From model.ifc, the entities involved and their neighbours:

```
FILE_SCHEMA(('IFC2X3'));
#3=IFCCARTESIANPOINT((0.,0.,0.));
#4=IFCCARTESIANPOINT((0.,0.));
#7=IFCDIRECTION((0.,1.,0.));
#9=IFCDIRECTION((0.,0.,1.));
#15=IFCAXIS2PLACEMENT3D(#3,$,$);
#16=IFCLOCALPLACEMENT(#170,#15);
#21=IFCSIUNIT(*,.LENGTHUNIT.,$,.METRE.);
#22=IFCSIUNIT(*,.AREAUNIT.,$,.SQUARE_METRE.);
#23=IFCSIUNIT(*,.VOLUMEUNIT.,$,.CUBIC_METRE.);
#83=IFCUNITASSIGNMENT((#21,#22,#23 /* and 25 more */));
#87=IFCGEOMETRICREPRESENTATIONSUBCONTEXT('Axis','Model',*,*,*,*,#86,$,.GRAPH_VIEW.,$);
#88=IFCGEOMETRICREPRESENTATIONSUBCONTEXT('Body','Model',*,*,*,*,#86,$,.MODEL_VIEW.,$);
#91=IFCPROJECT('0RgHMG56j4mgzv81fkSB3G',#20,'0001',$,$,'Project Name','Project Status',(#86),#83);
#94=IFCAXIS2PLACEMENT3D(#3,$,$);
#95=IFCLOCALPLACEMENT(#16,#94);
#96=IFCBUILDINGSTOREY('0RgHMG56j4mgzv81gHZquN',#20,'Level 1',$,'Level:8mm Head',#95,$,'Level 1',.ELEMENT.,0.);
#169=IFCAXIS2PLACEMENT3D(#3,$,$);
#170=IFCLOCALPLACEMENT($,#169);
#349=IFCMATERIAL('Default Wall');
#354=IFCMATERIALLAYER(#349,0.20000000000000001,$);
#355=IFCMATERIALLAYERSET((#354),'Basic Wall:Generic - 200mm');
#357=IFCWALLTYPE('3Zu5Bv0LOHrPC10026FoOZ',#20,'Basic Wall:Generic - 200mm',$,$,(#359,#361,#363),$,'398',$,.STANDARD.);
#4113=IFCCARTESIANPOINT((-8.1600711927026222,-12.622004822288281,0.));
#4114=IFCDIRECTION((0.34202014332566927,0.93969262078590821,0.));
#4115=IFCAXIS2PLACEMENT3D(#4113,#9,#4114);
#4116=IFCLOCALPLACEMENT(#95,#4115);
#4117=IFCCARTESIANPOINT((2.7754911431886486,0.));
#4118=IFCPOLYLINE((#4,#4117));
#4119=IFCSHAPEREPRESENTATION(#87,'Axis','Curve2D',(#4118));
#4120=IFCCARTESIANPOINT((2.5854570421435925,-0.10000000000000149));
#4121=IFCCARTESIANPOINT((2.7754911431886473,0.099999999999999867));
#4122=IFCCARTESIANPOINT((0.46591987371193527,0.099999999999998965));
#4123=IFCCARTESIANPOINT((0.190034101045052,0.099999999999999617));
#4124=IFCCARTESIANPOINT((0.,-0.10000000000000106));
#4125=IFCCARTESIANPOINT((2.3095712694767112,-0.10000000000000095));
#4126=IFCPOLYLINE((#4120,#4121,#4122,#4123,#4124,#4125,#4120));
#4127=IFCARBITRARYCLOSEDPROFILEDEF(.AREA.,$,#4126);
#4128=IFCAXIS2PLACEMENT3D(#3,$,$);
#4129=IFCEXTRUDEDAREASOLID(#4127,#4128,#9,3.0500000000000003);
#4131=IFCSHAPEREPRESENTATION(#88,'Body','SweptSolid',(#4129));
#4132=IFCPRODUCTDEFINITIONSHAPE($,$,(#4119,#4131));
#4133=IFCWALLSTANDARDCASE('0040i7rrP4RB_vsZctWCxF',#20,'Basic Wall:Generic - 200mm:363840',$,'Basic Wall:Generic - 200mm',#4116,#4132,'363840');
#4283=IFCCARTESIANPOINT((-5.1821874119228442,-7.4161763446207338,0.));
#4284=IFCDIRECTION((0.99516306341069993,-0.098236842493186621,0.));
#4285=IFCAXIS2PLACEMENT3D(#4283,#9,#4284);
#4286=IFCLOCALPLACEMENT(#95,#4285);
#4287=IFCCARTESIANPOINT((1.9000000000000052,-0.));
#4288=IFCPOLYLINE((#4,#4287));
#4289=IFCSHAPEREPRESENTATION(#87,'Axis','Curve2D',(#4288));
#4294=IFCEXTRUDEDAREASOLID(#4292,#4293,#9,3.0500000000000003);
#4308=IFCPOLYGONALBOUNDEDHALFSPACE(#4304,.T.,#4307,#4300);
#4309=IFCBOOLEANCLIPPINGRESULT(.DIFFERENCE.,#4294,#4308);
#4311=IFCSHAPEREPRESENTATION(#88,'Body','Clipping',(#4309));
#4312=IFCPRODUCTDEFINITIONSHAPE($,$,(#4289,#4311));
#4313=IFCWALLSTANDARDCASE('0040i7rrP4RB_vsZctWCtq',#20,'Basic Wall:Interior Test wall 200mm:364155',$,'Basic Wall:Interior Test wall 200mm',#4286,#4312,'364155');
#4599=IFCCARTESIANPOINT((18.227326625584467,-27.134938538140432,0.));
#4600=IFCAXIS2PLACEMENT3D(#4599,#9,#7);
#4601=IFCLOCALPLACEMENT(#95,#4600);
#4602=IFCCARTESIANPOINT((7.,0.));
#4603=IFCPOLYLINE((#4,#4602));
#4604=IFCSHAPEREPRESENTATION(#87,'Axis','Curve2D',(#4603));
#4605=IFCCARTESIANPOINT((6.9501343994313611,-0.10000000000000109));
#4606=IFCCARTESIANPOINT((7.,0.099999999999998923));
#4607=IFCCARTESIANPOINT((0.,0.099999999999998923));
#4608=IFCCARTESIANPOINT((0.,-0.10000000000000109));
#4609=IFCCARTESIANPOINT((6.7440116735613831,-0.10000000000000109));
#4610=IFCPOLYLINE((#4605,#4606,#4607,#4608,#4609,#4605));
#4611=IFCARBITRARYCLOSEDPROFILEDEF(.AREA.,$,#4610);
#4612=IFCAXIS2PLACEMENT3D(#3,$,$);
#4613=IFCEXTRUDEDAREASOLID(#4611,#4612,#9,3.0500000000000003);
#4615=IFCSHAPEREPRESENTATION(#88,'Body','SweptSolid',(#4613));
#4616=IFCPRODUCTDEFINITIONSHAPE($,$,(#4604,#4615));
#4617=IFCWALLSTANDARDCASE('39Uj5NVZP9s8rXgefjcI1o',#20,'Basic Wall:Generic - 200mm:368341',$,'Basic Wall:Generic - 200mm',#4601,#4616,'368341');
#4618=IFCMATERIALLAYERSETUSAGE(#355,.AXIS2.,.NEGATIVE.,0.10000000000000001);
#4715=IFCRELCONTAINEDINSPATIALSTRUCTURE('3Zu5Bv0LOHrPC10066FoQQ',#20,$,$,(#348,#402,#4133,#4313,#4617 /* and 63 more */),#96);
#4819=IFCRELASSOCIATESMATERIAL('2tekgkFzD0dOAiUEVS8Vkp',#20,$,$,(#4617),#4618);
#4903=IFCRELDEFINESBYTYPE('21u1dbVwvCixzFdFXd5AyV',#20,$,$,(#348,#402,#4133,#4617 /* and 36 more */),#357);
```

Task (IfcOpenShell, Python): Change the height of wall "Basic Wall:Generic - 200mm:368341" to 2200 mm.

```python
import ifcopenshell
import ifcopenshell.geom
import ifcopenshell.util.representation
import ifcopenshell.util.shape

model = ifcopenshell.open("model.ifc")
settings = ifcopenshell.geom.settings()


def volume(element):
    """Net volume in cubic metres, openings subtracted."""
    shape = ifcopenshell.geom.create_shape(settings, element)
    return ifcopenshell.util.shape.get_volume(shape.geometry)


wall = model.by_guid("39Uj5NVZP9s8rXgefjcI1o")
before = volume(wall)

body = ifcopenshell.util.representation.get_representation(wall, "Model", "Body")
solid = body.Items[0]
old_height = solid.Depth
solid.Depth = 2.2
after = volume(wall)

print(f"height {old_height:g} -> {solid.Depth:g}, volume {before:.3f} -> {after:.3f} m3")

model.write("model_updated.ifc")
```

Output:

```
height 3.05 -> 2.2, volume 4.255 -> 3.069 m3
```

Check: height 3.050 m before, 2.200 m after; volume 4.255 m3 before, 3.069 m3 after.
